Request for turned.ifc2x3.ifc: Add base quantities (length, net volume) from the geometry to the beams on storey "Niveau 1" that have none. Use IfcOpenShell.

First a look at what the model holds.

```python
import ifcopenshell
import ifcopenshell.util.element
import ifcopenshell.util.unit

model = ifcopenshell.open("turned.ifc2x3.ifc")
print(model.schema)
for unit_type in ("LENGTHUNIT", "AREAUNIT", "VOLUMEUNIT"):
    print(unit_type, ifcopenshell.util.unit.calculate_unit_scale(model, unit_type))
storey = next(s for s in model.by_type("IfcBuildingStorey") if s.Name == "Niveau 1")
beams = [e for e in ifcopenshell.util.element.get_decomposition(storey) if e.is_a("IfcBeam")]
for e in sorted(beams, key=lambda e: e.id()):
    print(e.id(), e.is_a(), e.Name, list(ifcopenshell.util.element.get_psets(e, qtos_only=True)), sep=" | ")
```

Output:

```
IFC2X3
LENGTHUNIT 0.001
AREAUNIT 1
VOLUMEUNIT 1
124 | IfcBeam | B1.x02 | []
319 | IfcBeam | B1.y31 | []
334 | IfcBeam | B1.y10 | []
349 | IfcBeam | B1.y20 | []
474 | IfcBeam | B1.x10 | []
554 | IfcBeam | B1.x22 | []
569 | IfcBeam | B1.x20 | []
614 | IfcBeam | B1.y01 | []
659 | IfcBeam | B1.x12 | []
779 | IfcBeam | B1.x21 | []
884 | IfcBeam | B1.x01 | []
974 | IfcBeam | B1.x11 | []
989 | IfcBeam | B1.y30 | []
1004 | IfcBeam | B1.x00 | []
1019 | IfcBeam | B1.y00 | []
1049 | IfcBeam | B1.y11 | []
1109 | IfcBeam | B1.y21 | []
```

```python
import ifcopenshell
import ifcopenshell.api.pset
import ifcopenshell.geom
import ifcopenshell.util.element
import ifcopenshell.util.shape
import ifcopenshell.util.unit

model = ifcopenshell.open("turned.ifc2x3.ifc")
unit_scale = ifcopenshell.util.unit.calculate_unit_scale(model)
volume_scale = ifcopenshell.util.unit.calculate_unit_scale(model, "VOLUMEUNIT")
settings = ifcopenshell.geom.settings()

storey = next(s for s in model.by_type("IfcBuildingStorey") if s.Name == "Niveau 1")
beams = [e for e in ifcopenshell.util.element.get_decomposition(storey) if e.is_a("IfcBeam")]

for e in sorted(beams, key=lambda e: e.id()):
    if ifcopenshell.util.element.get_psets(e, qtos_only=True, should_inherit=False):
        continue
    # Geometry comes back in metres, in the element's own axes.
    shape = ifcopenshell.geom.create_shape(settings, e)
    values = {
        "Length": ifcopenshell.util.shape.get_max_xyz(shape.geometry) / unit_scale,
        "NetVolume": ifcopenshell.util.shape.get_volume(shape.geometry) / volume_scale,
    }
    qto = ifcopenshell.api.pset.add_qto(model, product=e, name="BaseQuantities")
    ifcopenshell.api.pset.edit_qto(model, qto=qto, properties=values)
    print(e.id(), {k: round(v, 3) for k, v in values.items()})

model.write("turned.ifc2x3_updated.ifc")
```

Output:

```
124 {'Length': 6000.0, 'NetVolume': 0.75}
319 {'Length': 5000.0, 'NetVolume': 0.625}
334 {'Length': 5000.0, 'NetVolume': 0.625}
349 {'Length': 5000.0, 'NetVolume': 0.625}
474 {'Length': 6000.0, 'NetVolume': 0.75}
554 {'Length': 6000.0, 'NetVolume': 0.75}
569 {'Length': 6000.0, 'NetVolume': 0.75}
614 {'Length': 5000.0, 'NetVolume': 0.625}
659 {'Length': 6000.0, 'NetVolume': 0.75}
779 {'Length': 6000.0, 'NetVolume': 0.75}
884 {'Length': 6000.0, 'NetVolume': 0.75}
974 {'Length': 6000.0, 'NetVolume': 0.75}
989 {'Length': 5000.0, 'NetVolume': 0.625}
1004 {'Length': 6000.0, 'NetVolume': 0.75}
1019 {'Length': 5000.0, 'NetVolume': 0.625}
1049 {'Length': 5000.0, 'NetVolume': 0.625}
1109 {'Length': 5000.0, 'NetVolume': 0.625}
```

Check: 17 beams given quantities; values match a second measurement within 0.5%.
